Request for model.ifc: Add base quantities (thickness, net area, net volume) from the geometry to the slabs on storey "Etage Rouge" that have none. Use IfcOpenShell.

First a look at what the model holds.

```python
import ifcopenshell
import ifcopenshell.util.element
import ifcopenshell.util.unit

model = ifcopenshell.open("model.ifc")
print(model.schema)
for unit_type in ("LENGTHUNIT", "AREAUNIT", "VOLUMEUNIT"):
    print(unit_type, ifcopenshell.util.unit.calculate_unit_scale(model, unit_type))
storey = next(s for s in model.by_type("IfcBuildingStorey") if s.Name == "Etage Rouge")
slabs = [e for e in ifcopenshell.util.element.get_decomposition(storey) if e.is_a("IfcSlab")]
for e in sorted(slabs, key=lambda e: e.id()):
    print(e.id(), e.is_a(), e.Name, list(ifcopenshell.util.element.get_psets(e, qtos_only=True)), sep=" | ")
```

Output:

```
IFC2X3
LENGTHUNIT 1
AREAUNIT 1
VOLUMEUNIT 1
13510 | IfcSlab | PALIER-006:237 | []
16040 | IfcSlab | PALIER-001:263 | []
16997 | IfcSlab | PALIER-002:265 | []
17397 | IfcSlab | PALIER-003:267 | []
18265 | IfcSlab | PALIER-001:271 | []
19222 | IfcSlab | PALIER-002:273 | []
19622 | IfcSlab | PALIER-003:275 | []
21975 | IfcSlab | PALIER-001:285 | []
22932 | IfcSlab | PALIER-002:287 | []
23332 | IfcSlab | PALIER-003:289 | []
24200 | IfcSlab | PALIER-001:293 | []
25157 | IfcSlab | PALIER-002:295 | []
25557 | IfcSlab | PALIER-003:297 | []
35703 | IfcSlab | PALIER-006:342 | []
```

```python
import ifcopenshell
import ifcopenshell.api.pset
import ifcopenshell.geom
import ifcopenshell.util.element
import ifcopenshell.util.shape
import ifcopenshell.util.unit

model = ifcopenshell.open("model.ifc")
unit_scale = ifcopenshell.util.unit.calculate_unit_scale(model)
area_scale = ifcopenshell.util.unit.calculate_unit_scale(model, "AREAUNIT")
volume_scale = ifcopenshell.util.unit.calculate_unit_scale(model, "VOLUMEUNIT")
settings = ifcopenshell.geom.settings()

storey = next(s for s in model.by_type("IfcBuildingStorey") if s.Name == "Etage Rouge")
slabs = [e for e in ifcopenshell.util.element.get_decomposition(storey) if e.is_a("IfcSlab")]

for e in sorted(slabs, key=lambda e: e.id()):
    if ifcopenshell.util.element.get_psets(e, qtos_only=True, should_inherit=False):
        continue
    # Geometry comes back in metres, in the element's own axes.
    shape = ifcopenshell.geom.create_shape(settings, e)
    values = {
        "Width": ifcopenshell.util.shape.get_z(shape.geometry) / unit_scale,
        "NetArea": ifcopenshell.util.shape.get_footprint_area(shape.geometry) / area_scale,
        "NetVolume": ifcopenshell.util.shape.get_volume(shape.geometry) / volume_scale,
    }
    qto = ifcopenshell.api.pset.add_qto(model, product=e, name="BaseQuantities")
    ifcopenshell.api.pset.edit_qto(model, qto=qto, properties=values)
    print(e.id(), {k: round(v, 3) for k, v in values.items()})

model.write("model_rev.ifc")
```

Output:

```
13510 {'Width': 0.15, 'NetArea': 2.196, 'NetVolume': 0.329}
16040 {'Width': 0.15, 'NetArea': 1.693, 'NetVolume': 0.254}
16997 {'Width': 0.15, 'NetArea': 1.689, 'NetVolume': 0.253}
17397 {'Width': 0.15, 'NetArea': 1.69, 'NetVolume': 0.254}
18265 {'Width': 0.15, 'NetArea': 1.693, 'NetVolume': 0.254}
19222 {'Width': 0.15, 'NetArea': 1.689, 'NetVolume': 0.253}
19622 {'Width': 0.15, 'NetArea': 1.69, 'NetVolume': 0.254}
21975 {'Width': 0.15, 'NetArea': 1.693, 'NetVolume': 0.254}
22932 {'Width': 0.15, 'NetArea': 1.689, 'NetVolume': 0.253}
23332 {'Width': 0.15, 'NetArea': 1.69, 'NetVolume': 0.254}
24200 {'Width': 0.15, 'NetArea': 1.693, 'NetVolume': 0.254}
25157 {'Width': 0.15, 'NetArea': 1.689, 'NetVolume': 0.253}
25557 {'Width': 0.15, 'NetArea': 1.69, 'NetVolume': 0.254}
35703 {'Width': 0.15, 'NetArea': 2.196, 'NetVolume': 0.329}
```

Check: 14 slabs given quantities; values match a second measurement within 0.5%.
